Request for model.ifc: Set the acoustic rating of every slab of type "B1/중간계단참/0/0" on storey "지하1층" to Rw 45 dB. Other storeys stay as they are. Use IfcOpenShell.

First a look at what the model holds.

```python
import ifcopenshell
import ifcopenshell.util.element

model = ifcopenshell.open("model.ifc")
print(model.schema)
storey = next(s for s in model.by_type("IfcBuildingStorey") if s.Name == "지하1층")
slabs = [e for e in ifcopenshell.util.element.get_decomposition(storey) if e.is_a("IfcSlab")]
seen = {}
for e in slabs:
    element_type = ifcopenshell.util.element.get_type(e)
    key = (element_type.Name if element_type != e and element_type else None, ifcopenshell.util.element.get_pset(e, "Pset_SlabCommon", "AcousticRating"))
    seen[key] = seen.get(key, 0) + 1
for (name, value), count in sorted(seen.items(), key=str):
    print(count, "x", name, "|", value)
```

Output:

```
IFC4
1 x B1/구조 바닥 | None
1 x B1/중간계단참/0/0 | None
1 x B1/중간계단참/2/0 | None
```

```python
import ifcopenshell
import ifcopenshell.api.pset
import ifcopenshell.util.element

model = ifcopenshell.open("model.ifc")

storey = next(s for s in model.by_type("IfcBuildingStorey") if s.Name == "지하1층")
slabs = [e for e in ifcopenshell.util.element.get_decomposition(storey) if e.is_a("IfcSlab")]

count = 0
for e in slabs:
    element_type = ifcopenshell.util.element.get_type(e)
    if element_type in (None, e) or element_type.Name != "B1/중간계단참/0/0":
        continue
    # add_pset returns the element's existing set when there is one.
    pset = ifcopenshell.api.pset.add_pset(model, product=e, name="Pset_SlabCommon")
    ifcopenshell.api.pset.edit_pset(model, pset=pset, properties={"AcousticRating": "Rw 45 dB"})
    count += 1

print(count, "slabs updated")

model.write("model-out.ifc")
```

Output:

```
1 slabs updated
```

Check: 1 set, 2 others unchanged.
